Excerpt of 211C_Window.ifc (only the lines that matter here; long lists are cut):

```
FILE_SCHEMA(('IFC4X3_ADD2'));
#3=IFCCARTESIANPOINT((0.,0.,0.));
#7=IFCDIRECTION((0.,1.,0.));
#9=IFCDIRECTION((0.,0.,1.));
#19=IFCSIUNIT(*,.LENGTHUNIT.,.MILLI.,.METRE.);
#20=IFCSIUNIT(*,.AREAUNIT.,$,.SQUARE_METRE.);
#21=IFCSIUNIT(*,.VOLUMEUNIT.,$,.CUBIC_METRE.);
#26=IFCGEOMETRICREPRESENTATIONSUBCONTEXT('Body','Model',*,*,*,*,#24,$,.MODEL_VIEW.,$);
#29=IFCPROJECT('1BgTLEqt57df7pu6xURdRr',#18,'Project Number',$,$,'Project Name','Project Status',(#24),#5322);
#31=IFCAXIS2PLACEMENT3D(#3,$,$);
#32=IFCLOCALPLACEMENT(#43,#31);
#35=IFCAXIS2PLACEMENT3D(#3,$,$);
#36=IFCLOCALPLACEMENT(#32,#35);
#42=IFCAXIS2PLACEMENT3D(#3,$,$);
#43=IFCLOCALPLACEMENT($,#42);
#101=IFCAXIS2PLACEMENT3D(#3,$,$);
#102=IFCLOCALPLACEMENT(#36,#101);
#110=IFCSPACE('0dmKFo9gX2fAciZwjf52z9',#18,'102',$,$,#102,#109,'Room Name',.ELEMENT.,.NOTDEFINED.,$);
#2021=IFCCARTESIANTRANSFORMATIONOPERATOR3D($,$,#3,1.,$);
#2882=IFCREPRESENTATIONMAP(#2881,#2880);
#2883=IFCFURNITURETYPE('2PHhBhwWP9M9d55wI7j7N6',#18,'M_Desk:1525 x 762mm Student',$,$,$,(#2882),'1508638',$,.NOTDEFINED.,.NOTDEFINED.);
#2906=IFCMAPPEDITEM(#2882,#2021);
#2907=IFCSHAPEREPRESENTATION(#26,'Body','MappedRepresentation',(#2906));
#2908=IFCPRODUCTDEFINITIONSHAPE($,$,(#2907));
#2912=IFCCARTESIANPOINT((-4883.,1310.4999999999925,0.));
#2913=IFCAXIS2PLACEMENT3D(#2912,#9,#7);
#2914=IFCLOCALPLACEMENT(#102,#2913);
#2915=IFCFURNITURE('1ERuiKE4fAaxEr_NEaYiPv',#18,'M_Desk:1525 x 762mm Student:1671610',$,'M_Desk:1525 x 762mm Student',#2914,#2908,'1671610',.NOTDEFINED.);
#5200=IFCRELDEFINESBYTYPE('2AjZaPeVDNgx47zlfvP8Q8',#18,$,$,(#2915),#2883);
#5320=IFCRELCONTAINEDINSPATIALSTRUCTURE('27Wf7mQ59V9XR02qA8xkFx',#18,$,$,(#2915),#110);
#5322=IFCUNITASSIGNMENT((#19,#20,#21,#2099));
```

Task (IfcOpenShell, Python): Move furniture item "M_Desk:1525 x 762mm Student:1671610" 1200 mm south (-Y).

```python
import ifcopenshell
import ifcopenshell.api.geometry
import ifcopenshell.util.placement

model = ifcopenshell.open("211C_Window.ifc")

item = model.by_id(2915)
matrix = ifcopenshell.util.placement.get_local_placement(item.ObjectPlacement)
matrix[1, 3] -= 1200.0
ifcopenshell.api.geometry.edit_object_placement(model, product=item, matrix=matrix, is_si=False)

print(ifcopenshell.util.placement.get_local_placement(item.ObjectPlacement).round(3) + 0.0)

model.write("211C_Window_rev.ifc")
```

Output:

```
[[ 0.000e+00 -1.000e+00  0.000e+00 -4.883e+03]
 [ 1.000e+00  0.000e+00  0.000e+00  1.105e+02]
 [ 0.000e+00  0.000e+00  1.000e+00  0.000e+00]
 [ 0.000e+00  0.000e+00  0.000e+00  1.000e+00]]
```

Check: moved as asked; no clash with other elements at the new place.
